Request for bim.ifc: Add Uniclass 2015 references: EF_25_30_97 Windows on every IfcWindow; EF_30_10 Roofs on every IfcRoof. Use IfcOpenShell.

First a look at what the model holds.

```python
import ifcopenshell

model = ifcopenshell.open("bim.ifc")
print(model.schema)
print("classifications:", [c.Name for c in model.by_type("IfcClassification")])
for ifc_class in ("IfcDoor", "IfcRoof", "IfcStair", "IfcWall", "IfcWindow"):
    print(ifc_class, len(model.by_type(ifc_class)))
```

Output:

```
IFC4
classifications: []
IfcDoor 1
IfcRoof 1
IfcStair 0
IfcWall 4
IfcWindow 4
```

```python
import ifcopenshell
import ifcopenshell.api.classification

model = ifcopenshell.open("bim.ifc")

system = ifcopenshell.api.classification.add_classification(model, classification="Uniclass 2015")

codes = {
    "IfcWindow": ("EF_25_30_97", "Windows"),
    "IfcRoof": ("EF_30_10", "Roofs"),
}
for ifc_class, (code, name) in codes.items():
    products = model.by_type(ifc_class)
    ifcopenshell.api.classification.add_reference(
        model, products=products, classification=system, identification=code, name=name
    )
    print(code, len(products))

model.write("bim_updated.ifc")
```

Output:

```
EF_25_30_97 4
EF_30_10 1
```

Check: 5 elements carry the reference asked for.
